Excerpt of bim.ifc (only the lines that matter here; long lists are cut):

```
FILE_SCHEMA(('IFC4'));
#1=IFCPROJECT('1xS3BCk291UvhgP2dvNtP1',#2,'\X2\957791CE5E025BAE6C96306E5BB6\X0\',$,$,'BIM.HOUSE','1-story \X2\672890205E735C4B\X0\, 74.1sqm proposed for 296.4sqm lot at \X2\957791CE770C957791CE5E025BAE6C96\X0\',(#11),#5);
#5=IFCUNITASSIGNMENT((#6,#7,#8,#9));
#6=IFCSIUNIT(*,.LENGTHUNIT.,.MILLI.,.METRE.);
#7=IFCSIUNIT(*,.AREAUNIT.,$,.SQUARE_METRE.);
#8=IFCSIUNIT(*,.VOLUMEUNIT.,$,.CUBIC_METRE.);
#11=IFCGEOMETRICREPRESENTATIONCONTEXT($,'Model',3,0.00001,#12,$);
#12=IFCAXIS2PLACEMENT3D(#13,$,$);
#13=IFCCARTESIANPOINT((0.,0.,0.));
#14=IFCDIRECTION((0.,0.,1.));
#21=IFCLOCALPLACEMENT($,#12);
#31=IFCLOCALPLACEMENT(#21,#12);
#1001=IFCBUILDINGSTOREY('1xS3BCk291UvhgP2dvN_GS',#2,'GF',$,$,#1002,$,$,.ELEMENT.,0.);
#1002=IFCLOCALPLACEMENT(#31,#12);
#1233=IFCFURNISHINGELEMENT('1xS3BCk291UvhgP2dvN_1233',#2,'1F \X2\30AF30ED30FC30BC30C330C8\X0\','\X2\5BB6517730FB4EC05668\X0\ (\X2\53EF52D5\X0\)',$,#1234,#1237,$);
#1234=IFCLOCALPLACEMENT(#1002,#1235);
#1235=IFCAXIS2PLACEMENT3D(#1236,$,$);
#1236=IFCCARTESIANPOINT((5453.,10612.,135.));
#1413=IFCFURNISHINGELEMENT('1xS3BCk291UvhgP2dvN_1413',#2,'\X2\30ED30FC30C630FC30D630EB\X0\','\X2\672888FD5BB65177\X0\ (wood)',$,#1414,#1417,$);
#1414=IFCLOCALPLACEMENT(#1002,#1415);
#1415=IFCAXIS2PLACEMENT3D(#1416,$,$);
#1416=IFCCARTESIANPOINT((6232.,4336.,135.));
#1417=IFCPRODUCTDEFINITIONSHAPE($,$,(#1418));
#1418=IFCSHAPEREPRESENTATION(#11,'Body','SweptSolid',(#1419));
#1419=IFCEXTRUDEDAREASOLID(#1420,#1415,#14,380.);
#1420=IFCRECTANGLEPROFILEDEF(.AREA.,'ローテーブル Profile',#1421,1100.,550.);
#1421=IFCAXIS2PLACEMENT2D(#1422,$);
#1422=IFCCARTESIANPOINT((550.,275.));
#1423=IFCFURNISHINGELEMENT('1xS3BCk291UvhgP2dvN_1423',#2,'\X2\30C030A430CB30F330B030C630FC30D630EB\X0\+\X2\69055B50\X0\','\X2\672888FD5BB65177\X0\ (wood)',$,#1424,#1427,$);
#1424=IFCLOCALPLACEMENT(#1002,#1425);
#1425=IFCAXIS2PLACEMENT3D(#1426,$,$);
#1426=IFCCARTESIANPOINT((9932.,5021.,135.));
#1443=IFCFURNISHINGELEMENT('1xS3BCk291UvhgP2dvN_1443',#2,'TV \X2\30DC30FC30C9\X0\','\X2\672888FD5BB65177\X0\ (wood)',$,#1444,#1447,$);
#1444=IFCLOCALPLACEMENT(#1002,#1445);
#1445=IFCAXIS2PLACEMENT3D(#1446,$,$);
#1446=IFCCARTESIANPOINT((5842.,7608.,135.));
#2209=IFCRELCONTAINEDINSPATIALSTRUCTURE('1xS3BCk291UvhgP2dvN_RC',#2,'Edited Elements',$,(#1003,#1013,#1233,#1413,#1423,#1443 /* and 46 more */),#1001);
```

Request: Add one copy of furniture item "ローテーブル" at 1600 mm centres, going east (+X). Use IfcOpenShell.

```python
import numpy as np
import ifcopenshell
import ifcopenshell.api.geometry
import ifcopenshell.api.root
import ifcopenshell.util.element
import ifcopenshell.util.placement
import ifcopenshell.util.unit

model = ifcopenshell.open("bim.ifc")
unit_scale = ifcopenshell.util.unit.calculate_unit_scale(model)


def reuse_history(source, copy):
    """copy_class also copies each property set's owner history, people and application; keep the originals."""
    for rel in copy.IsDefinedBy:
        if rel.is_a("IfcRelDefinesByProperties") and (history := rel.RelatingPropertyDefinition.OwnerHistory):
            rel.RelatingPropertyDefinition.OwnerHistory = source.OwnerHistory
            ifcopenshell.util.element.remove_deep2(model, history)


source = model.by_guid("1xS3BCk291UvhgP2dvN_1413")
base = ifcopenshell.util.placement.get_local_placement(source.ObjectPlacement)
step = np.array([1.0, 0.0, 0.0]) * 1.6 / unit_scale

for i in range(1, 2):
    copy = ifcopenshell.api.root.copy_class(model, product=source)
    copy.Representation = ifcopenshell.util.element.copy_deep(
        model, source.Representation, exclude=["IfcGeometricRepresentationContext", "IfcRepresentationMap"]
    )
    reuse_history(source, copy)
    matrix = base.copy()
    matrix[:3, 3] += i * step
    print("added at", matrix[:3, 3].round(3) + 0.0)
    ifcopenshell.api.geometry.edit_object_placement(model, product=copy, matrix=matrix, is_si=False)

model.write("bim_rev.ifc")
```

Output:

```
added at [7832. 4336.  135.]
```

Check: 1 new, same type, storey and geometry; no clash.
